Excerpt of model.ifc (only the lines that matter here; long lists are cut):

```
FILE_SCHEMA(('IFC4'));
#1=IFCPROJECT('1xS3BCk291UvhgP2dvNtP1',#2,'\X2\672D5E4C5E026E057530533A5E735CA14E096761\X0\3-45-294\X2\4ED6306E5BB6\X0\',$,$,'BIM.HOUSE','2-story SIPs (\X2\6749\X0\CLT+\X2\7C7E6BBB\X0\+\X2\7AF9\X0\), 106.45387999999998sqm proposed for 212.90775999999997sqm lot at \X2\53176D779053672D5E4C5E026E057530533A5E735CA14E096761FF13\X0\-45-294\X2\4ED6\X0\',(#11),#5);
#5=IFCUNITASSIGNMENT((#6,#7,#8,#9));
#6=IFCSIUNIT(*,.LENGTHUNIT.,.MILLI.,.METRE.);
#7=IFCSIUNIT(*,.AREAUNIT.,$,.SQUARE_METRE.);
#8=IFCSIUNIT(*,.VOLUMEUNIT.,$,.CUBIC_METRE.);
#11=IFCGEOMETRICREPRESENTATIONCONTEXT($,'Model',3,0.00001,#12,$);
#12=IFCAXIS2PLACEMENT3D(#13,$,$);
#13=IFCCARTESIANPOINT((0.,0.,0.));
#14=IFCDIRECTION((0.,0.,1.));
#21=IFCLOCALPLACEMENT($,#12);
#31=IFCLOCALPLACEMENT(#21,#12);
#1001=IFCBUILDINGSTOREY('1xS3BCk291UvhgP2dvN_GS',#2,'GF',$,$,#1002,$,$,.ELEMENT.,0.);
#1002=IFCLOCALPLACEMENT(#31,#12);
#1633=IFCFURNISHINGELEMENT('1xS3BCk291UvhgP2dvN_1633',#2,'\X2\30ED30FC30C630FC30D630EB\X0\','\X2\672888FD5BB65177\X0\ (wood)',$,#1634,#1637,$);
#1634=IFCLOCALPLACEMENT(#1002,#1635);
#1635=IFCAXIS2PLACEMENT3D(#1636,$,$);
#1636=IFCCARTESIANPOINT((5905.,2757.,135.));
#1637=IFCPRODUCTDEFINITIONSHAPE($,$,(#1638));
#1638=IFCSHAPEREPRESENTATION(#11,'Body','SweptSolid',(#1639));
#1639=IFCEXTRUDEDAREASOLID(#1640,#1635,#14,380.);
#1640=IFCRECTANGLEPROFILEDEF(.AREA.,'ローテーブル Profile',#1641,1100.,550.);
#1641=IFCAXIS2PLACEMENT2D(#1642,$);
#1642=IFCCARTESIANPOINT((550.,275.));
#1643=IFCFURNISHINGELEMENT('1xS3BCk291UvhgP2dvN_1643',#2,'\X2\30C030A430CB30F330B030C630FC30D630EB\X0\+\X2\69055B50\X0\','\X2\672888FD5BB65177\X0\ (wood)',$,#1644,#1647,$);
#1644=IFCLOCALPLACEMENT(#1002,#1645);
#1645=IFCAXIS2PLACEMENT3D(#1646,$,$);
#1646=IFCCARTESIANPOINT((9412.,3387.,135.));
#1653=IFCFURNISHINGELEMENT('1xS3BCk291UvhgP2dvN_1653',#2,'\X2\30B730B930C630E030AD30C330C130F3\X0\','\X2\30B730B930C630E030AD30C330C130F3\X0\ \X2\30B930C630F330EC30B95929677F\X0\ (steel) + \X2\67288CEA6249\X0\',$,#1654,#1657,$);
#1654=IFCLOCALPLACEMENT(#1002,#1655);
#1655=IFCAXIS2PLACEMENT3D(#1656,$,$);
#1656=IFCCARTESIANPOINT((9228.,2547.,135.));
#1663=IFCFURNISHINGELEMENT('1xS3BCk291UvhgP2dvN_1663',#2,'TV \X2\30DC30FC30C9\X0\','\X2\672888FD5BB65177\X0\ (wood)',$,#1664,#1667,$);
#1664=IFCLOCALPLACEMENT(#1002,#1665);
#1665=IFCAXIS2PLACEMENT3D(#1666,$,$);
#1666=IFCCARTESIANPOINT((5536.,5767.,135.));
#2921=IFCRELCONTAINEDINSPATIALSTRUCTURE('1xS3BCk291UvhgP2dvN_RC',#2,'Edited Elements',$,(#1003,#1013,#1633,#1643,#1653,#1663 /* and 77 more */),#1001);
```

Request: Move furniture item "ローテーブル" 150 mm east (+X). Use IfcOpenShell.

```python
import ifcopenshell
import ifcopenshell.api.geometry
import ifcopenshell.util.placement
import ifcopenshell.util.unit

model = ifcopenshell.open("model.ifc")
unit_scale = ifcopenshell.util.unit.calculate_unit_scale(model)

item = model.by_guid("1xS3BCk291UvhgP2dvN_1633")
matrix = ifcopenshell.util.placement.get_local_placement(item.ObjectPlacement)
matrix[0, 3] += 0.15 / unit_scale
ifcopenshell.api.geometry.edit_object_placement(model, product=item, matrix=matrix, is_si=False)

print(ifcopenshell.util.placement.get_local_placement(item.ObjectPlacement).round(3) + 0.0)

model.write("model_updated.ifc")
```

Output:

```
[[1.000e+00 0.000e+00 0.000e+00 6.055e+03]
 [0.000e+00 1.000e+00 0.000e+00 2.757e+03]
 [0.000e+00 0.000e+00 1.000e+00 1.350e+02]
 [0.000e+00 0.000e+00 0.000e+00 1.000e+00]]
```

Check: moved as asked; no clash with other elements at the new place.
